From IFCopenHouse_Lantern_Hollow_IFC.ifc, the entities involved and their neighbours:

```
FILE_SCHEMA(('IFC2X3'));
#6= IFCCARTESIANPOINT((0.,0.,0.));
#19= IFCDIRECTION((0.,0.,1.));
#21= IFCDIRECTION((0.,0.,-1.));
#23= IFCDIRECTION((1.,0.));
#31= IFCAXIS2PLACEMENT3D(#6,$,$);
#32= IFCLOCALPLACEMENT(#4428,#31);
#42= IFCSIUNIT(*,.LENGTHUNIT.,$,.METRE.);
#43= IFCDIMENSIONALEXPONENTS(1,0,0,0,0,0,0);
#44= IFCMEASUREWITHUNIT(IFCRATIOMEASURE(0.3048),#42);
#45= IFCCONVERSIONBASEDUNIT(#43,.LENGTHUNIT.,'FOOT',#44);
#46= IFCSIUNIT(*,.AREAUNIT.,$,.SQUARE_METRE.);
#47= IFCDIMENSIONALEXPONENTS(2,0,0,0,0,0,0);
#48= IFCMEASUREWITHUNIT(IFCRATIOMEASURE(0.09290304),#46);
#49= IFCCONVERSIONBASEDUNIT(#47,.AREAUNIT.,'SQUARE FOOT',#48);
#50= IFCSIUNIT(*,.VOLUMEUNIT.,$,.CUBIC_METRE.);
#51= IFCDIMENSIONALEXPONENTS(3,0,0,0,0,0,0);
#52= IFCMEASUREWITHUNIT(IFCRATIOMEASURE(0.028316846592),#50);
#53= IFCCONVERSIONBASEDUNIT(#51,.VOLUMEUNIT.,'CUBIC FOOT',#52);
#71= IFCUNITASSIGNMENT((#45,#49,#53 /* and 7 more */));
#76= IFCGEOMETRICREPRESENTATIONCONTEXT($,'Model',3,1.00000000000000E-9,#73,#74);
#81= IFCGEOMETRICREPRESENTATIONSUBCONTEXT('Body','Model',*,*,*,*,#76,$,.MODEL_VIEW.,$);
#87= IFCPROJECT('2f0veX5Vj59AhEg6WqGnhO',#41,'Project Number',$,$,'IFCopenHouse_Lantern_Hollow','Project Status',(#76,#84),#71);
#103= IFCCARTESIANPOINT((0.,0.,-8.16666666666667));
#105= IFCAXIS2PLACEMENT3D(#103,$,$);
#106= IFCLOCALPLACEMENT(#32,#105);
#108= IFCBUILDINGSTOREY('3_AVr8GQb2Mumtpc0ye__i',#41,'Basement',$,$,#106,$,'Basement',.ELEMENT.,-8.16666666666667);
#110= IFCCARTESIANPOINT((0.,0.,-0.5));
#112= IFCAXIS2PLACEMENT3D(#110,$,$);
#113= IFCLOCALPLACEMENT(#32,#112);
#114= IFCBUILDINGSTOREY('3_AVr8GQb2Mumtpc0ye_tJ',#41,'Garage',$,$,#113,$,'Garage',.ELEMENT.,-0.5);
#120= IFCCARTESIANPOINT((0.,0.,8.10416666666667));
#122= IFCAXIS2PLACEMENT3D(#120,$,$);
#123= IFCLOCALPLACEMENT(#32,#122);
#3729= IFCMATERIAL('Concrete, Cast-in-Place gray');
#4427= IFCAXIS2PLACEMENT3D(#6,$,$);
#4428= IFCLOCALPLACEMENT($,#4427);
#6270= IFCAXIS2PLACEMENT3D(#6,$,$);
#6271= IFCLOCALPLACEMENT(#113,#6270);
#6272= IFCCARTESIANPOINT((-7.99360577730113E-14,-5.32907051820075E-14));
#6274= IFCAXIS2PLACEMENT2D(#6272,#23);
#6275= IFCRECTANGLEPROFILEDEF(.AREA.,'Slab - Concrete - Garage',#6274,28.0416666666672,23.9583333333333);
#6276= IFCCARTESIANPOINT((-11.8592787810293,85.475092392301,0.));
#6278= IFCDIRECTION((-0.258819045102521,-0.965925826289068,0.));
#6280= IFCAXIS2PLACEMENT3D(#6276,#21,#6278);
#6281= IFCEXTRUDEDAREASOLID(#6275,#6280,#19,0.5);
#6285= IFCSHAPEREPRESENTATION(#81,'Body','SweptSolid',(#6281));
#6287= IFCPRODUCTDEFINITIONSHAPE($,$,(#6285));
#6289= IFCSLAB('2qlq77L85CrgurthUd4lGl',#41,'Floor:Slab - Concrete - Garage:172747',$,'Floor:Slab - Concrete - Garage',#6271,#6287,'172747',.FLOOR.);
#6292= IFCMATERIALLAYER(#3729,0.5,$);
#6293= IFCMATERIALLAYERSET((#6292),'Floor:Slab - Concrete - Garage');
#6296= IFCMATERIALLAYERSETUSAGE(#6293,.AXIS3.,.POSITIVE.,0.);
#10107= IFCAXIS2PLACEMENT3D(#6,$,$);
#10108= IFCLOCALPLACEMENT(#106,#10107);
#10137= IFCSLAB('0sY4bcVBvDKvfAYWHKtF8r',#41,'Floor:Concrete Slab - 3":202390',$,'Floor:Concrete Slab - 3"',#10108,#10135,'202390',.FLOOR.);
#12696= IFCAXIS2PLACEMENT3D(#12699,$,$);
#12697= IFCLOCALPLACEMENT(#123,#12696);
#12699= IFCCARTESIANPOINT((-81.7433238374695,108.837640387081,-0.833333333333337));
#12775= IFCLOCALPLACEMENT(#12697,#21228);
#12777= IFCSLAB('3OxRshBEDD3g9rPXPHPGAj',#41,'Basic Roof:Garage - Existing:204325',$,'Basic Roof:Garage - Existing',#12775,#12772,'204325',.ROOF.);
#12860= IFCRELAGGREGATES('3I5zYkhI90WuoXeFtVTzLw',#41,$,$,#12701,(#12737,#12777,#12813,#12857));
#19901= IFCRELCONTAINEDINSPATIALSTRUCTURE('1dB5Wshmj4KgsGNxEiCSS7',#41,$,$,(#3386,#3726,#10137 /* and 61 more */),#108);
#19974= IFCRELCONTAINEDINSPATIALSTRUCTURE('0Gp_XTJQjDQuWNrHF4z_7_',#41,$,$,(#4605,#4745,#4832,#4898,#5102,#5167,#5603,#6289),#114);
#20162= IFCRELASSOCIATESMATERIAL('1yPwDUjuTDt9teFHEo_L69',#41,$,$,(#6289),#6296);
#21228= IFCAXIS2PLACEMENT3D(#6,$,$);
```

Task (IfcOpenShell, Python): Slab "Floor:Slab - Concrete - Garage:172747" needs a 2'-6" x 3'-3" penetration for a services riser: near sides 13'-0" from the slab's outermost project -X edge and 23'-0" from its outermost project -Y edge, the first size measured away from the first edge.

```python
import numpy as np
import ifcopenshell
import ifcopenshell.api.feature
import ifcopenshell.api.geometry
import ifcopenshell.api.root
import ifcopenshell.geom
import ifcopenshell.util.placement
import ifcopenshell.util.representation
import ifcopenshell.util.shape
import ifcopenshell.util.unit

model = ifcopenshell.open("IFCopenHouse_Lantern_Hollow_IFC.ifc")
unit_scale = ifcopenshell.util.unit.calculate_unit_scale(model)
settings = ifcopenshell.geom.settings()


def volume(element):
    """Net volume in cubic metres, openings subtracted."""
    shape = ifcopenshell.geom.create_shape(settings, element)
    return ifcopenshell.util.shape.get_volume(shape.geometry)


slab = model.by_id(6289)
before = volume(slab)

# Extent in the slab's own axes, in metres. The edges named are its -X and -Y sides.
slab_shape = ifcopenshell.geom.create_shape(settings, slab)
vertices = ifcopenshell.util.shape.get_vertices(slab_shape.geometry)
x_min, y_min, bottom = vertices.min(axis=0)
top = vertices[:, 2].max()

opening = ifcopenshell.api.root.create_entity(model, ifc_class="IfcOpeningElement", name="Services riser opening")
context = ifcopenshell.util.representation.get_context(model, "Model", "Body", "MODEL_VIEW")
width, depth = 0.762, 0.9906
outline = [(0.0, 0.0), (width, 0.0), (width, depth), (0.0, depth), (0.0, 0.0)]
# Overshoot both faces by 50 mm so the cut is clean.
shape = ifcopenshell.api.geometry.add_slab_representation(
    model, context=context, depth=top - bottom + 0.1, polyline=outline
)
ifcopenshell.api.geometry.assign_representation(model, product=opening, representation=shape)

matrix = ifcopenshell.util.placement.get_local_placement(slab.ObjectPlacement)
matrix[:, 3] = matrix @ np.append(np.array([x_min + 3.9624, y_min + 7.0104, bottom - 0.05]) / unit_scale, 1.0)
ifcopenshell.api.geometry.edit_object_placement(model, product=opening, matrix=matrix, is_si=False)
ifcopenshell.api.feature.add_feature(model, feature=opening, element=slab)

after = volume(slab)

print(f"slab volume {before:.3f} -> {after:.3f} m3")

model.write("IFCopenHouse_Lantern_Hollow_IFC_updated.ifc")
```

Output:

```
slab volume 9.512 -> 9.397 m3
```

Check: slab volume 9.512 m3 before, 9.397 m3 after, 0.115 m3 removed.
